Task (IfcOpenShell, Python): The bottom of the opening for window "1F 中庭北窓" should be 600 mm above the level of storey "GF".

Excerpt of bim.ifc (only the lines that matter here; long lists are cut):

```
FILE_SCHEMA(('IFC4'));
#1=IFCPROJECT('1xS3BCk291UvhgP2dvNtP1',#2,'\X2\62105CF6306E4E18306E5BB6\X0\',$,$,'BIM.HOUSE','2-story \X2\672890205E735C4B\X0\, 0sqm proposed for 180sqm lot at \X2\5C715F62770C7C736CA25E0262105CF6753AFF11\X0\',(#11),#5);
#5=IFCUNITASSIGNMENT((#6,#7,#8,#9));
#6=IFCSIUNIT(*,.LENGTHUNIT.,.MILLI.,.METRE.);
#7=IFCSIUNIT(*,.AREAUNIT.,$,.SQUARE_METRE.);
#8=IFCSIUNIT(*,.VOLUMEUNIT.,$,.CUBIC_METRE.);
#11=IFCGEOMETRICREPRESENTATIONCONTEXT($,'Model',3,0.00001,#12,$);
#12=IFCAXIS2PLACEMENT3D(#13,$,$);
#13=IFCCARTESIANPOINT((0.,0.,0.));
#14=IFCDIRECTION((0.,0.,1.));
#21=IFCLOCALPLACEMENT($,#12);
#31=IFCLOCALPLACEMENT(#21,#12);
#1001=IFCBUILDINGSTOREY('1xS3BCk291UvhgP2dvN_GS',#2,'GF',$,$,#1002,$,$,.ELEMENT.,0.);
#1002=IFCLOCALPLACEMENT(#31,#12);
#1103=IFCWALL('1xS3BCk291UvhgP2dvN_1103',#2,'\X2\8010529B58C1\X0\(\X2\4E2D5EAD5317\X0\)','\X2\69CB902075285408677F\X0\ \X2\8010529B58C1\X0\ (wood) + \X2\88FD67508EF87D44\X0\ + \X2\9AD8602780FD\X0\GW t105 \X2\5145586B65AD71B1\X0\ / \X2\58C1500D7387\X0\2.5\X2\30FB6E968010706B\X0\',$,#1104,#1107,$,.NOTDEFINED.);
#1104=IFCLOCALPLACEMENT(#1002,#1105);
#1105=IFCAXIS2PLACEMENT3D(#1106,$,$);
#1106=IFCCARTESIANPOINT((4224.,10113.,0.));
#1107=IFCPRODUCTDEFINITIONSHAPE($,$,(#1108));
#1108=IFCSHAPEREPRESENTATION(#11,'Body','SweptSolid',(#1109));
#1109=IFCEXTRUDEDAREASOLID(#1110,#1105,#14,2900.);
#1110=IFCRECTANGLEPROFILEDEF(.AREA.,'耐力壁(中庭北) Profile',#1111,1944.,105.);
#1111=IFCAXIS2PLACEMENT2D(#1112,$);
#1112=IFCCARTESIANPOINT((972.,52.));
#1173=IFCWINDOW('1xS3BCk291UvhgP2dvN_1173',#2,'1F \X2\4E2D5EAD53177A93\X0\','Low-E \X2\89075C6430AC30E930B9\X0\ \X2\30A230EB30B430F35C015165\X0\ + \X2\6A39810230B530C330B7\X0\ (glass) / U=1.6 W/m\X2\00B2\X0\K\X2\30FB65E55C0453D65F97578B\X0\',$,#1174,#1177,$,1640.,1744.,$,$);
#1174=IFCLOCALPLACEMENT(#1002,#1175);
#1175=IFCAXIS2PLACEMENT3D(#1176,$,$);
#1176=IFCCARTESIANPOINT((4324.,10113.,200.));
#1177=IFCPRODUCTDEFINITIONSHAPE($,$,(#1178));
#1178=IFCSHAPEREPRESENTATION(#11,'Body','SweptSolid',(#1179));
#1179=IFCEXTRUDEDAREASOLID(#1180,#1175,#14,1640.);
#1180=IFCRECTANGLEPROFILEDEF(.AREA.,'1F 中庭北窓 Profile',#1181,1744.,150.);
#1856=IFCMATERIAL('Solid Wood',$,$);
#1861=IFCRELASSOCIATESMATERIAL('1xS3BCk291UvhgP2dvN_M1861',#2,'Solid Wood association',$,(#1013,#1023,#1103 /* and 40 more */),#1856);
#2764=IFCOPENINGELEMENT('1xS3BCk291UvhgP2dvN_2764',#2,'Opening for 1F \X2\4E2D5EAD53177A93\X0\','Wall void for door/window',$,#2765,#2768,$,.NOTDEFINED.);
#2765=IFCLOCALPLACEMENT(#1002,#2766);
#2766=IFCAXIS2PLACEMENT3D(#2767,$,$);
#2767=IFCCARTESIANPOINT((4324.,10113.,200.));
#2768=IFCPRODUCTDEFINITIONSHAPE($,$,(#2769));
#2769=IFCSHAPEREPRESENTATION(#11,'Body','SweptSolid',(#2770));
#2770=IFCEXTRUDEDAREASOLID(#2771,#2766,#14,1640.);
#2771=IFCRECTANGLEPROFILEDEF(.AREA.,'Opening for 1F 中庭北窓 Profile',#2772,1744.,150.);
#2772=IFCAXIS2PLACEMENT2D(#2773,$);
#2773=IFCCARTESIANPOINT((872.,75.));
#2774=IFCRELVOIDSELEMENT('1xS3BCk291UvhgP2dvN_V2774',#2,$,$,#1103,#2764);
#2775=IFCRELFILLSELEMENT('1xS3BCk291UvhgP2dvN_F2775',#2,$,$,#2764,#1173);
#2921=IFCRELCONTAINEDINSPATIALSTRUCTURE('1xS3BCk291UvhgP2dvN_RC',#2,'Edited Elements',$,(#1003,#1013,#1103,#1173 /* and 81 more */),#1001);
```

```python
import numpy as np
import ifcopenshell
import ifcopenshell.api.geometry
import ifcopenshell.geom
import ifcopenshell.util.element
import ifcopenshell.util.placement
import ifcopenshell.util.shape
import ifcopenshell.util.unit

model = ifcopenshell.open("bim.ifc")
unit_scale = ifcopenshell.util.unit.calculate_unit_scale(model)

window = model.by_guid("1xS3BCk291UvhgP2dvN_1173")
opening = window.FillsVoids[0].RelatingOpeningElement
storey = ifcopenshell.util.element.get_container(window, ifc_class="IfcBuildingStorey")
level = ifcopenshell.util.placement.get_local_placement(storey.ObjectPlacement)[2, 3]

# The opening's origin need not be at the sill, so measure its lowest point.
shape = ifcopenshell.geom.create_shape(ifcopenshell.geom.settings(), opening)
bottom = ifcopenshell.util.shape.get_shape_bottom_elevation(shape, shape.geometry) / unit_scale
dz = level + 0.6 / unit_scale - bottom

shift = np.array([0.0, 0.0, dz])
# The window is not placed relative to its opening, so move both.
for product in (opening, window):
    matrix = ifcopenshell.util.placement.get_local_placement(product.ObjectPlacement)
    matrix[:3, 3] += shift
    ifcopenshell.api.geometry.edit_object_placement(model, product=product, matrix=matrix, is_si=False)

print(f"moved by {dz * unit_scale:+.3f} m")

model.write("bim-out.ifc")
```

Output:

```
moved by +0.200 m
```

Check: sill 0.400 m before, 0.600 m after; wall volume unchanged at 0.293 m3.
